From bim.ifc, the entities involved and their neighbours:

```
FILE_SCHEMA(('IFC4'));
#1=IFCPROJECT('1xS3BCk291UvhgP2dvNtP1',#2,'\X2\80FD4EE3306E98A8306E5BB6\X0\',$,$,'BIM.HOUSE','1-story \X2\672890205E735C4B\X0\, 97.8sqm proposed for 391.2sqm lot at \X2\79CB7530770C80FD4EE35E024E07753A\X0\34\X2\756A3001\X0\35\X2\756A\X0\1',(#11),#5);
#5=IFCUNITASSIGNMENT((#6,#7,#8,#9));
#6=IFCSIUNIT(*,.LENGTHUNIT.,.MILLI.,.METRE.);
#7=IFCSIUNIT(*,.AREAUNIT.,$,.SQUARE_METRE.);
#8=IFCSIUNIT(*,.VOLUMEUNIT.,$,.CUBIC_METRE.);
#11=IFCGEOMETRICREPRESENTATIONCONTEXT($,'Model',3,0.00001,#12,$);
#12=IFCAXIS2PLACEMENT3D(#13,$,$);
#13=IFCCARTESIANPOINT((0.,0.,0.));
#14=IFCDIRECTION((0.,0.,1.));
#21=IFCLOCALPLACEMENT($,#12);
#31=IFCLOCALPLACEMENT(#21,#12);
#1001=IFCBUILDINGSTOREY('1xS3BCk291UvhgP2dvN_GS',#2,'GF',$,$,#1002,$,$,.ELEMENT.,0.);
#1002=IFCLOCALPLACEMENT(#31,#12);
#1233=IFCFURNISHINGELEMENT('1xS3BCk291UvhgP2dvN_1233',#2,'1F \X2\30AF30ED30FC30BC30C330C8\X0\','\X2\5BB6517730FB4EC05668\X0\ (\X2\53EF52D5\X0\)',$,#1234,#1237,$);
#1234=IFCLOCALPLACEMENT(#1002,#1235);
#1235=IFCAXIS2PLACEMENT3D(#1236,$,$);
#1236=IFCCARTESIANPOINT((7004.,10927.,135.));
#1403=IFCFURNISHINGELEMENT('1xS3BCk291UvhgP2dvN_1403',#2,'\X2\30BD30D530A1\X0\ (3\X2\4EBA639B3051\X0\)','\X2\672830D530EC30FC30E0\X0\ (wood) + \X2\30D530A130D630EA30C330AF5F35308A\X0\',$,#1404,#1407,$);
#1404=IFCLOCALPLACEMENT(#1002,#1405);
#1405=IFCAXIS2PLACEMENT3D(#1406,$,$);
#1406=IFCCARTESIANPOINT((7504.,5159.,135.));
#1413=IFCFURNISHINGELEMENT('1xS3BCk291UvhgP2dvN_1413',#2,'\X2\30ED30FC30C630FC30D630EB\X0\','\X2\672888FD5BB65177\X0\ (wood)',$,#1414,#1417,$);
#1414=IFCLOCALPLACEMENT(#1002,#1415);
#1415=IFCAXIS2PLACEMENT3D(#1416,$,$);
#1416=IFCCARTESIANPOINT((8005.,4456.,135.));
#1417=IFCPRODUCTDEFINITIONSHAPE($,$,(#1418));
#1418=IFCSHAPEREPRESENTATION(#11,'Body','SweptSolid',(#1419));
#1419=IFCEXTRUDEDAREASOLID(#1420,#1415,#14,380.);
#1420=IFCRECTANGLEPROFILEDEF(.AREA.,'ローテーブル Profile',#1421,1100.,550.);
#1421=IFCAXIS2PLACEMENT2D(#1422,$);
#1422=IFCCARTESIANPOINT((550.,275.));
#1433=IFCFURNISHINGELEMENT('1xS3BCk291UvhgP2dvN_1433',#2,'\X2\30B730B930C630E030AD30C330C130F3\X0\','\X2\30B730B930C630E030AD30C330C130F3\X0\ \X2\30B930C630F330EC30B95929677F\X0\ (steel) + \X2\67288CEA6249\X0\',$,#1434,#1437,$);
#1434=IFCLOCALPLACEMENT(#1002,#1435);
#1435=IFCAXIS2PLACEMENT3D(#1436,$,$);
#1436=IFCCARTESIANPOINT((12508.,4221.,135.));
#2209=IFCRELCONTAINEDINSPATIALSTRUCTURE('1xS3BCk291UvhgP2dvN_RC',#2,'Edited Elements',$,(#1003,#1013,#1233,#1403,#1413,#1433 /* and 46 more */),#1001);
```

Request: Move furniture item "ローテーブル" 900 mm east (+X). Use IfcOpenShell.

```python
import ifcopenshell
import ifcopenshell.api.geometry
import ifcopenshell.util.placement

model = ifcopenshell.open("bim.ifc")

item = model.by_guid("1xS3BCk291UvhgP2dvN_1413")
matrix = ifcopenshell.util.placement.get_local_placement(item.ObjectPlacement)
matrix[0, 3] += 900.0
ifcopenshell.api.geometry.edit_object_placement(model, product=item, matrix=matrix, is_si=False)

print(ifcopenshell.util.placement.get_local_placement(item.ObjectPlacement).round(3) + 0.0)

model.write("bim_v2.ifc")
```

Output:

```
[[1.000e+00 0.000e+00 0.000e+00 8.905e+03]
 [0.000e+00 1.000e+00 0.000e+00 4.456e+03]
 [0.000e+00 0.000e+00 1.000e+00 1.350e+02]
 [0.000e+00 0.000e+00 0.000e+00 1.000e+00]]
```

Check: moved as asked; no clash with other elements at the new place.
